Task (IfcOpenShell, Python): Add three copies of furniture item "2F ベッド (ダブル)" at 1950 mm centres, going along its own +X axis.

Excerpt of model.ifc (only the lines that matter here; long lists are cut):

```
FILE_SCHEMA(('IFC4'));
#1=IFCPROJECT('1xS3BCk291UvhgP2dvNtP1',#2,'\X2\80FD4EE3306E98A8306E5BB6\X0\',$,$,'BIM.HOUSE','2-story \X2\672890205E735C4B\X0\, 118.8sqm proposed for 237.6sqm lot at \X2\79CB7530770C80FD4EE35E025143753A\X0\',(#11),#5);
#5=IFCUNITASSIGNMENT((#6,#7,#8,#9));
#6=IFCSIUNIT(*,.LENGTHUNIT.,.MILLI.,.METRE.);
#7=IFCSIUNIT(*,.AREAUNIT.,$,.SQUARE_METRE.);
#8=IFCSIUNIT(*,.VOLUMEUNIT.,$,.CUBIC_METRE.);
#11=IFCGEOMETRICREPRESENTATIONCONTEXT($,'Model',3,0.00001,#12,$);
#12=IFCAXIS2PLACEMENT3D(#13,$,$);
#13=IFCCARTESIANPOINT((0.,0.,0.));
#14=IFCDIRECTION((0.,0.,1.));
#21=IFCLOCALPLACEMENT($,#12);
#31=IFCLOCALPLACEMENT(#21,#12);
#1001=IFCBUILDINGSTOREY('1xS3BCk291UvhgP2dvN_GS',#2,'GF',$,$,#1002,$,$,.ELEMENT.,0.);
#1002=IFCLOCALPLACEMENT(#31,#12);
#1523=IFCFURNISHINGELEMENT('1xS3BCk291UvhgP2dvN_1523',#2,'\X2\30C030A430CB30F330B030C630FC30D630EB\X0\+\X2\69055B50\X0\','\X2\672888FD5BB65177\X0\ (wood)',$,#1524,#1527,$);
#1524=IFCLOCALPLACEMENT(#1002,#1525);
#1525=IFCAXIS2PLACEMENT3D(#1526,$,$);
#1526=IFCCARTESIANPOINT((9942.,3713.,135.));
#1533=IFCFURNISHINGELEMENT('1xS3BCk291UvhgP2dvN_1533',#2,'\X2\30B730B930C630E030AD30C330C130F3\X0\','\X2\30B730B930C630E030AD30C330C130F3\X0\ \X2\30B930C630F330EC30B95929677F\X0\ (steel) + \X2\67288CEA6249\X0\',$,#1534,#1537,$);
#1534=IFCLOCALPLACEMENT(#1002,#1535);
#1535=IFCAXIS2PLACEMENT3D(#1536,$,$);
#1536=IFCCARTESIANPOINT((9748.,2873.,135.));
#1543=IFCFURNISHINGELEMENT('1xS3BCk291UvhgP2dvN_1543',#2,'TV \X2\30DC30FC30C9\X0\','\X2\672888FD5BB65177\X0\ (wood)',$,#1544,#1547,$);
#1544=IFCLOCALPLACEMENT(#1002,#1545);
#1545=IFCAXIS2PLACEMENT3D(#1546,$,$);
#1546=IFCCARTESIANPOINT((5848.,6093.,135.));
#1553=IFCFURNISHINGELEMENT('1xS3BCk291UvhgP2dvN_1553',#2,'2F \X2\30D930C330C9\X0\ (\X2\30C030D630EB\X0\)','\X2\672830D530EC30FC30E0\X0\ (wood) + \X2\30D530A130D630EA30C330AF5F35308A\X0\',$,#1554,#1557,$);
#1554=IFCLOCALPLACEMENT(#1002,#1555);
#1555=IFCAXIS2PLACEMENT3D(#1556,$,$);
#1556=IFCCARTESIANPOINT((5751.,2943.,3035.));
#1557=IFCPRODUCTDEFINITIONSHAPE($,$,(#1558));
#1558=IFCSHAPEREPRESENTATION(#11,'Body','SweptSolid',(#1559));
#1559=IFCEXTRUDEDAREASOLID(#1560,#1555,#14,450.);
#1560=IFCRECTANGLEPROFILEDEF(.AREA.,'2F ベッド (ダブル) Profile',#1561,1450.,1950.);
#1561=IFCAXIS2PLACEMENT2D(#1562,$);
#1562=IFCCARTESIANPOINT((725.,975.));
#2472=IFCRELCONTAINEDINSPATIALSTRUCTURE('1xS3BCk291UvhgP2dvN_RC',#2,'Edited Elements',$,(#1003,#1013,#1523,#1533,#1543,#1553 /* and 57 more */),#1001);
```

```python
import ifcopenshell
import ifcopenshell.api.geometry
import ifcopenshell.api.root
import ifcopenshell.util.element
import ifcopenshell.util.placement

model = ifcopenshell.open("model.ifc")


def reuse_history(source, copy):
    """copy_class also copies each property set's owner history, people and application; keep the originals."""
    for rel in copy.IsDefinedBy:
        if rel.is_a("IfcRelDefinesByProperties") and (history := rel.RelatingPropertyDefinition.OwnerHistory):
            rel.RelatingPropertyDefinition.OwnerHistory = source.OwnerHistory
            ifcopenshell.util.element.remove_deep2(model, history)


source = model.by_id(1553)
base = ifcopenshell.util.placement.get_local_placement(source.ObjectPlacement)
step = base[:3, 0] * 1950.0

for i in range(1, 4):
    copy = ifcopenshell.api.root.copy_class(model, product=source)
    copy.Representation = ifcopenshell.util.element.copy_deep(
        model, source.Representation, exclude=["IfcGeometricRepresentationContext", "IfcRepresentationMap"]
    )
    reuse_history(source, copy)
    matrix = base.copy()
    matrix[:3, 3] += i * step
    print("added at", matrix[:3, 3].round(3) + 0.0)
    ifcopenshell.api.geometry.edit_object_placement(model, product=copy, matrix=matrix, is_si=False)

model.write("model_updated.ifc")
```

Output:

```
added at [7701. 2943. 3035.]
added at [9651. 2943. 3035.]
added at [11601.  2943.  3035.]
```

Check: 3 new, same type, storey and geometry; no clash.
